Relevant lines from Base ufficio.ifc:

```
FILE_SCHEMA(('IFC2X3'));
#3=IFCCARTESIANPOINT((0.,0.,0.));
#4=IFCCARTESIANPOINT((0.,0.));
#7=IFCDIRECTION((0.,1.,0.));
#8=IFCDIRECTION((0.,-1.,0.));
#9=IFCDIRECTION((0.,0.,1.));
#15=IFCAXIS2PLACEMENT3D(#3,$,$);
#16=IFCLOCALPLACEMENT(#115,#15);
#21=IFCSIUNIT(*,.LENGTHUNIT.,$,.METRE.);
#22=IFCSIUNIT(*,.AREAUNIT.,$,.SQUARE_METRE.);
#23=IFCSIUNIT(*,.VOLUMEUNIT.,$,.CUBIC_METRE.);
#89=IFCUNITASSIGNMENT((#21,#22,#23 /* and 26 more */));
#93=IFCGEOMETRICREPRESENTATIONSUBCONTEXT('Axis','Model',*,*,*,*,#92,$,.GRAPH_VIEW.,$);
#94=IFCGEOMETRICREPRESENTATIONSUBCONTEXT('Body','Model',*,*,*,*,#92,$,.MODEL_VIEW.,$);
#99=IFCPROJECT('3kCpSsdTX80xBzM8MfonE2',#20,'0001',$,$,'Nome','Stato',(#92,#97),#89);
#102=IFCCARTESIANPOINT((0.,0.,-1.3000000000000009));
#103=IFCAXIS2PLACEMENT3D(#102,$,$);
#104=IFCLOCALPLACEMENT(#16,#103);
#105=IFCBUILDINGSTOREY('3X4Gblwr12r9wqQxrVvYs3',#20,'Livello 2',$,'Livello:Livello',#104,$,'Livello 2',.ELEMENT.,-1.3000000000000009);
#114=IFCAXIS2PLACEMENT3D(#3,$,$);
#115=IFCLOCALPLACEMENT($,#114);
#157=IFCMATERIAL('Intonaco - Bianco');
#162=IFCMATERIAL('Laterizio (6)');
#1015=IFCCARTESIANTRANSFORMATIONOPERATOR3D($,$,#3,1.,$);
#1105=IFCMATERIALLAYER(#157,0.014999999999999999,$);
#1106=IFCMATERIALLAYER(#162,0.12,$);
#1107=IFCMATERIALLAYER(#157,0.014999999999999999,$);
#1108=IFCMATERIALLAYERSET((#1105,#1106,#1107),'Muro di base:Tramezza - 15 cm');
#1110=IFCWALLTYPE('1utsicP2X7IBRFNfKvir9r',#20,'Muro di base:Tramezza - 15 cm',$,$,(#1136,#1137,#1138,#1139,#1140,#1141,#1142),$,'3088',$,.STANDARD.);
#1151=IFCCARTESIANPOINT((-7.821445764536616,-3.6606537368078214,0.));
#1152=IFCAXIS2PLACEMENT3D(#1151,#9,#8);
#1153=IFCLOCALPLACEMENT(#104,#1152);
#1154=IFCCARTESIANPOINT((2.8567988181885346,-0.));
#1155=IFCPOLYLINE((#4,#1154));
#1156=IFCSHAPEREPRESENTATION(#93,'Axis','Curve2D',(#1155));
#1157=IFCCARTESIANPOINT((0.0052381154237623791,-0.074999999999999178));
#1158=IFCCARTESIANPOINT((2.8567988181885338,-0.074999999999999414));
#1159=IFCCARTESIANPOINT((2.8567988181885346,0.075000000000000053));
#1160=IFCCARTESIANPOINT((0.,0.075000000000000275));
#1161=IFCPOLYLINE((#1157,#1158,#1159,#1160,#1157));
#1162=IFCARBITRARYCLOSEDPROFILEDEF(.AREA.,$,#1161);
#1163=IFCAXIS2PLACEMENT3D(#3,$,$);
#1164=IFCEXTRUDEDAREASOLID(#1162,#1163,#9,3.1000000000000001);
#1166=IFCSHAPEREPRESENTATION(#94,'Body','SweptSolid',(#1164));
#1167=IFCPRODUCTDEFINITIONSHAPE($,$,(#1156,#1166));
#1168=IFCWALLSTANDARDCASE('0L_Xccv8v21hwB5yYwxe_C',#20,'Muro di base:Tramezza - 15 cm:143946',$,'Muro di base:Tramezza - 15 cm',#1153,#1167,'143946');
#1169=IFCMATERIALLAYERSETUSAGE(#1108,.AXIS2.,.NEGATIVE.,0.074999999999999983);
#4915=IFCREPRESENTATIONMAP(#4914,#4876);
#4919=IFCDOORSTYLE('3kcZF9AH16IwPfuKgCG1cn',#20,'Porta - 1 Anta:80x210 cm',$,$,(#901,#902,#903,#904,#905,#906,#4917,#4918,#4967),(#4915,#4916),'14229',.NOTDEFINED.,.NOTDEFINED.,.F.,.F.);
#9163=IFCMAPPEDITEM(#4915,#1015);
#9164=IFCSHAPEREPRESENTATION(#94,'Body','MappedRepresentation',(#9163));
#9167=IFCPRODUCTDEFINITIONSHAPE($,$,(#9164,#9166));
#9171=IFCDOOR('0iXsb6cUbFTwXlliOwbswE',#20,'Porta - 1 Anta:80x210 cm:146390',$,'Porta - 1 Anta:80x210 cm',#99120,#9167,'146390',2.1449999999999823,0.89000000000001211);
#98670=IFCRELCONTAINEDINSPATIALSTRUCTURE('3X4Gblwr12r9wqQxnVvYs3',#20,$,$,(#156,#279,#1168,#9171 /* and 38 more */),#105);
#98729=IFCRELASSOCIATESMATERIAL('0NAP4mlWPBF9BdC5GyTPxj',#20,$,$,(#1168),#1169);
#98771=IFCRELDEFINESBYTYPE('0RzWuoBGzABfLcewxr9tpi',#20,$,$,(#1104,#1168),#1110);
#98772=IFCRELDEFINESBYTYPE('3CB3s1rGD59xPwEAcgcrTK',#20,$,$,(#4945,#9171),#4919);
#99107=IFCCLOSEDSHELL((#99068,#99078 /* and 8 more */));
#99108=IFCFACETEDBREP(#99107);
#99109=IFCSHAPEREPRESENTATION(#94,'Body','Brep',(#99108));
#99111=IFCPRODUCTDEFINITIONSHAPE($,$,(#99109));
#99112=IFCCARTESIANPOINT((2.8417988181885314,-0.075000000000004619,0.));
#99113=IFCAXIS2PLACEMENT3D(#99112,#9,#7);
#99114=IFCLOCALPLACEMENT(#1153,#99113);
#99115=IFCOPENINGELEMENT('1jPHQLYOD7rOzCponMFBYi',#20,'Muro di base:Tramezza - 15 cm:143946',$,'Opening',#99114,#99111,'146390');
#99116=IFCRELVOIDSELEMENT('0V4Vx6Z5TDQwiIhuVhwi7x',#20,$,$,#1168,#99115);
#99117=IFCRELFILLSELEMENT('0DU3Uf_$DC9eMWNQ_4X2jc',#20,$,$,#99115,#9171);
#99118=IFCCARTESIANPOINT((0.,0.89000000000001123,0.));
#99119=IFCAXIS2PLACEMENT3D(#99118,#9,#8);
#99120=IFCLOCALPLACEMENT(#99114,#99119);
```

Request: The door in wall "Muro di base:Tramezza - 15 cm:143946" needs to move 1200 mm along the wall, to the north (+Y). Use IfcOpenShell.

```python
import ifcopenshell
import ifcopenshell.api.geometry
import ifcopenshell.util.placement
import ifcopenshell.util.unit

model = ifcopenshell.open("Base ufficio.ifc")
unit_scale = ifcopenshell.util.unit.calculate_unit_scale(model)

door = model.by_guid("0iXsb6cUbFTwXlliOwbswE")
opening = door.FillsVoids[0].RelatingOpeningElement
wall = opening.VoidsElements[0].RelatingBuildingElement

wall_matrix = ifcopenshell.util.placement.get_local_placement(wall.ObjectPlacement)
shift = wall_matrix[:3, 0] * -1.2 / unit_scale
before = ifcopenshell.util.placement.get_local_placement(door.ObjectPlacement)[:3, 3].copy()

# The door is placed relative to its opening, so it follows when the opening moves.
matrix = ifcopenshell.util.placement.get_local_placement(opening.ObjectPlacement)
matrix[:3, 3] += shift
ifcopenshell.api.geometry.edit_object_placement(
    model, product=opening, matrix=matrix, is_si=False, should_transform_children=True
)

after = ifcopenshell.util.placement.get_local_placement(door.ObjectPlacement)[:3, 3]
print("door moved by", (after - before).round(3) + 0.0)

model.write("Base ufficio-out.ifc")
```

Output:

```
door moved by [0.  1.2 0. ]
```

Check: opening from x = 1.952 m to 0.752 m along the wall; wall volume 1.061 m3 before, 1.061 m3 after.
